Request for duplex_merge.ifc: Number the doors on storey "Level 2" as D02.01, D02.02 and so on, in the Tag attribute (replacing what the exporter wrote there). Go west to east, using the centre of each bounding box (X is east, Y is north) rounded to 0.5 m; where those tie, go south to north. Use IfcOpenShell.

First a look at what the model holds.

```python
import ifcopenshell
import ifcopenshell.util.element
import ifcopenshell.util.placement

model = ifcopenshell.open("duplex_merge.ifc")
print(model.schema)
storey = next(s for s in model.by_type("IfcBuildingStorey") if s.Name == "Level 2")
doors = [e for e in ifcopenshell.util.element.get_decomposition(storey) if e.is_a("IfcDoor")]
for e in sorted(doors, key=lambda e: e.id()):
    origin = ifcopenshell.util.placement.get_local_placement(e.ObjectPlacement)[:3, 3]
    print(e.id(), e.Tag, e.Name, origin.round(2) + 0.0, sep=" | ")
```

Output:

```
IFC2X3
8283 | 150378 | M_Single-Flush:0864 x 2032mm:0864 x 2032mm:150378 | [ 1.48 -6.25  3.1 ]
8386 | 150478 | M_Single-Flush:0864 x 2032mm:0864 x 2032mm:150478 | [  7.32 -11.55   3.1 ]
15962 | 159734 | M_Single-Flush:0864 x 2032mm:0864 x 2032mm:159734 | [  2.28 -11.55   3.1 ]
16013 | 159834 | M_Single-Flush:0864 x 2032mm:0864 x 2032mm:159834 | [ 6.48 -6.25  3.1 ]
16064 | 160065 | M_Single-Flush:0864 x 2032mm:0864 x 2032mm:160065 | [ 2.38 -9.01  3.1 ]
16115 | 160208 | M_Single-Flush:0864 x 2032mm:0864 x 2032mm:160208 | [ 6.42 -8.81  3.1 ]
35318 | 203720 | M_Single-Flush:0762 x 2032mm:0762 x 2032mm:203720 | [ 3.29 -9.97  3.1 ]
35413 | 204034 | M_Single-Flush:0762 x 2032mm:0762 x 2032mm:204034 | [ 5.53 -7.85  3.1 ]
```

```python
import ifcopenshell
import ifcopenshell.geom
import ifcopenshell.util.element
import ifcopenshell.util.shape

model = ifcopenshell.open("duplex_merge.ifc")
settings = ifcopenshell.geom.settings()
settings.set("use-world-coords", True)


def centre(element):
    shape = ifcopenshell.geom.create_shape(settings, element)
    return ifcopenshell.util.shape.get_bbox_centroid(shape.geometry)


storey = next(s for s in model.by_type("IfcBuildingStorey") if s.Name == "Level 2")
doors = [e for e in ifcopenshell.util.element.get_decomposition(storey) if e.is_a("IfcDoor")]

# Insertion points can sit at a corner or the storey origin, so sort by the geometry (in metres).
centres = {e: centre(e) for e in doors}
doors.sort(key=lambda e: (round(centres[e][0] / 0.5), centres[e][1]))

for i, e in enumerate(doors, start=1):
    number = f"D02.{i:02d}"
    e.Tag = number
    print(e.id(), number)

model.write("duplex_merge_rev.ifc")
```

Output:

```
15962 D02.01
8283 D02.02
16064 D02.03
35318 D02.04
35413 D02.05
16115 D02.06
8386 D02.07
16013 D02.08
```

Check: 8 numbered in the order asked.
